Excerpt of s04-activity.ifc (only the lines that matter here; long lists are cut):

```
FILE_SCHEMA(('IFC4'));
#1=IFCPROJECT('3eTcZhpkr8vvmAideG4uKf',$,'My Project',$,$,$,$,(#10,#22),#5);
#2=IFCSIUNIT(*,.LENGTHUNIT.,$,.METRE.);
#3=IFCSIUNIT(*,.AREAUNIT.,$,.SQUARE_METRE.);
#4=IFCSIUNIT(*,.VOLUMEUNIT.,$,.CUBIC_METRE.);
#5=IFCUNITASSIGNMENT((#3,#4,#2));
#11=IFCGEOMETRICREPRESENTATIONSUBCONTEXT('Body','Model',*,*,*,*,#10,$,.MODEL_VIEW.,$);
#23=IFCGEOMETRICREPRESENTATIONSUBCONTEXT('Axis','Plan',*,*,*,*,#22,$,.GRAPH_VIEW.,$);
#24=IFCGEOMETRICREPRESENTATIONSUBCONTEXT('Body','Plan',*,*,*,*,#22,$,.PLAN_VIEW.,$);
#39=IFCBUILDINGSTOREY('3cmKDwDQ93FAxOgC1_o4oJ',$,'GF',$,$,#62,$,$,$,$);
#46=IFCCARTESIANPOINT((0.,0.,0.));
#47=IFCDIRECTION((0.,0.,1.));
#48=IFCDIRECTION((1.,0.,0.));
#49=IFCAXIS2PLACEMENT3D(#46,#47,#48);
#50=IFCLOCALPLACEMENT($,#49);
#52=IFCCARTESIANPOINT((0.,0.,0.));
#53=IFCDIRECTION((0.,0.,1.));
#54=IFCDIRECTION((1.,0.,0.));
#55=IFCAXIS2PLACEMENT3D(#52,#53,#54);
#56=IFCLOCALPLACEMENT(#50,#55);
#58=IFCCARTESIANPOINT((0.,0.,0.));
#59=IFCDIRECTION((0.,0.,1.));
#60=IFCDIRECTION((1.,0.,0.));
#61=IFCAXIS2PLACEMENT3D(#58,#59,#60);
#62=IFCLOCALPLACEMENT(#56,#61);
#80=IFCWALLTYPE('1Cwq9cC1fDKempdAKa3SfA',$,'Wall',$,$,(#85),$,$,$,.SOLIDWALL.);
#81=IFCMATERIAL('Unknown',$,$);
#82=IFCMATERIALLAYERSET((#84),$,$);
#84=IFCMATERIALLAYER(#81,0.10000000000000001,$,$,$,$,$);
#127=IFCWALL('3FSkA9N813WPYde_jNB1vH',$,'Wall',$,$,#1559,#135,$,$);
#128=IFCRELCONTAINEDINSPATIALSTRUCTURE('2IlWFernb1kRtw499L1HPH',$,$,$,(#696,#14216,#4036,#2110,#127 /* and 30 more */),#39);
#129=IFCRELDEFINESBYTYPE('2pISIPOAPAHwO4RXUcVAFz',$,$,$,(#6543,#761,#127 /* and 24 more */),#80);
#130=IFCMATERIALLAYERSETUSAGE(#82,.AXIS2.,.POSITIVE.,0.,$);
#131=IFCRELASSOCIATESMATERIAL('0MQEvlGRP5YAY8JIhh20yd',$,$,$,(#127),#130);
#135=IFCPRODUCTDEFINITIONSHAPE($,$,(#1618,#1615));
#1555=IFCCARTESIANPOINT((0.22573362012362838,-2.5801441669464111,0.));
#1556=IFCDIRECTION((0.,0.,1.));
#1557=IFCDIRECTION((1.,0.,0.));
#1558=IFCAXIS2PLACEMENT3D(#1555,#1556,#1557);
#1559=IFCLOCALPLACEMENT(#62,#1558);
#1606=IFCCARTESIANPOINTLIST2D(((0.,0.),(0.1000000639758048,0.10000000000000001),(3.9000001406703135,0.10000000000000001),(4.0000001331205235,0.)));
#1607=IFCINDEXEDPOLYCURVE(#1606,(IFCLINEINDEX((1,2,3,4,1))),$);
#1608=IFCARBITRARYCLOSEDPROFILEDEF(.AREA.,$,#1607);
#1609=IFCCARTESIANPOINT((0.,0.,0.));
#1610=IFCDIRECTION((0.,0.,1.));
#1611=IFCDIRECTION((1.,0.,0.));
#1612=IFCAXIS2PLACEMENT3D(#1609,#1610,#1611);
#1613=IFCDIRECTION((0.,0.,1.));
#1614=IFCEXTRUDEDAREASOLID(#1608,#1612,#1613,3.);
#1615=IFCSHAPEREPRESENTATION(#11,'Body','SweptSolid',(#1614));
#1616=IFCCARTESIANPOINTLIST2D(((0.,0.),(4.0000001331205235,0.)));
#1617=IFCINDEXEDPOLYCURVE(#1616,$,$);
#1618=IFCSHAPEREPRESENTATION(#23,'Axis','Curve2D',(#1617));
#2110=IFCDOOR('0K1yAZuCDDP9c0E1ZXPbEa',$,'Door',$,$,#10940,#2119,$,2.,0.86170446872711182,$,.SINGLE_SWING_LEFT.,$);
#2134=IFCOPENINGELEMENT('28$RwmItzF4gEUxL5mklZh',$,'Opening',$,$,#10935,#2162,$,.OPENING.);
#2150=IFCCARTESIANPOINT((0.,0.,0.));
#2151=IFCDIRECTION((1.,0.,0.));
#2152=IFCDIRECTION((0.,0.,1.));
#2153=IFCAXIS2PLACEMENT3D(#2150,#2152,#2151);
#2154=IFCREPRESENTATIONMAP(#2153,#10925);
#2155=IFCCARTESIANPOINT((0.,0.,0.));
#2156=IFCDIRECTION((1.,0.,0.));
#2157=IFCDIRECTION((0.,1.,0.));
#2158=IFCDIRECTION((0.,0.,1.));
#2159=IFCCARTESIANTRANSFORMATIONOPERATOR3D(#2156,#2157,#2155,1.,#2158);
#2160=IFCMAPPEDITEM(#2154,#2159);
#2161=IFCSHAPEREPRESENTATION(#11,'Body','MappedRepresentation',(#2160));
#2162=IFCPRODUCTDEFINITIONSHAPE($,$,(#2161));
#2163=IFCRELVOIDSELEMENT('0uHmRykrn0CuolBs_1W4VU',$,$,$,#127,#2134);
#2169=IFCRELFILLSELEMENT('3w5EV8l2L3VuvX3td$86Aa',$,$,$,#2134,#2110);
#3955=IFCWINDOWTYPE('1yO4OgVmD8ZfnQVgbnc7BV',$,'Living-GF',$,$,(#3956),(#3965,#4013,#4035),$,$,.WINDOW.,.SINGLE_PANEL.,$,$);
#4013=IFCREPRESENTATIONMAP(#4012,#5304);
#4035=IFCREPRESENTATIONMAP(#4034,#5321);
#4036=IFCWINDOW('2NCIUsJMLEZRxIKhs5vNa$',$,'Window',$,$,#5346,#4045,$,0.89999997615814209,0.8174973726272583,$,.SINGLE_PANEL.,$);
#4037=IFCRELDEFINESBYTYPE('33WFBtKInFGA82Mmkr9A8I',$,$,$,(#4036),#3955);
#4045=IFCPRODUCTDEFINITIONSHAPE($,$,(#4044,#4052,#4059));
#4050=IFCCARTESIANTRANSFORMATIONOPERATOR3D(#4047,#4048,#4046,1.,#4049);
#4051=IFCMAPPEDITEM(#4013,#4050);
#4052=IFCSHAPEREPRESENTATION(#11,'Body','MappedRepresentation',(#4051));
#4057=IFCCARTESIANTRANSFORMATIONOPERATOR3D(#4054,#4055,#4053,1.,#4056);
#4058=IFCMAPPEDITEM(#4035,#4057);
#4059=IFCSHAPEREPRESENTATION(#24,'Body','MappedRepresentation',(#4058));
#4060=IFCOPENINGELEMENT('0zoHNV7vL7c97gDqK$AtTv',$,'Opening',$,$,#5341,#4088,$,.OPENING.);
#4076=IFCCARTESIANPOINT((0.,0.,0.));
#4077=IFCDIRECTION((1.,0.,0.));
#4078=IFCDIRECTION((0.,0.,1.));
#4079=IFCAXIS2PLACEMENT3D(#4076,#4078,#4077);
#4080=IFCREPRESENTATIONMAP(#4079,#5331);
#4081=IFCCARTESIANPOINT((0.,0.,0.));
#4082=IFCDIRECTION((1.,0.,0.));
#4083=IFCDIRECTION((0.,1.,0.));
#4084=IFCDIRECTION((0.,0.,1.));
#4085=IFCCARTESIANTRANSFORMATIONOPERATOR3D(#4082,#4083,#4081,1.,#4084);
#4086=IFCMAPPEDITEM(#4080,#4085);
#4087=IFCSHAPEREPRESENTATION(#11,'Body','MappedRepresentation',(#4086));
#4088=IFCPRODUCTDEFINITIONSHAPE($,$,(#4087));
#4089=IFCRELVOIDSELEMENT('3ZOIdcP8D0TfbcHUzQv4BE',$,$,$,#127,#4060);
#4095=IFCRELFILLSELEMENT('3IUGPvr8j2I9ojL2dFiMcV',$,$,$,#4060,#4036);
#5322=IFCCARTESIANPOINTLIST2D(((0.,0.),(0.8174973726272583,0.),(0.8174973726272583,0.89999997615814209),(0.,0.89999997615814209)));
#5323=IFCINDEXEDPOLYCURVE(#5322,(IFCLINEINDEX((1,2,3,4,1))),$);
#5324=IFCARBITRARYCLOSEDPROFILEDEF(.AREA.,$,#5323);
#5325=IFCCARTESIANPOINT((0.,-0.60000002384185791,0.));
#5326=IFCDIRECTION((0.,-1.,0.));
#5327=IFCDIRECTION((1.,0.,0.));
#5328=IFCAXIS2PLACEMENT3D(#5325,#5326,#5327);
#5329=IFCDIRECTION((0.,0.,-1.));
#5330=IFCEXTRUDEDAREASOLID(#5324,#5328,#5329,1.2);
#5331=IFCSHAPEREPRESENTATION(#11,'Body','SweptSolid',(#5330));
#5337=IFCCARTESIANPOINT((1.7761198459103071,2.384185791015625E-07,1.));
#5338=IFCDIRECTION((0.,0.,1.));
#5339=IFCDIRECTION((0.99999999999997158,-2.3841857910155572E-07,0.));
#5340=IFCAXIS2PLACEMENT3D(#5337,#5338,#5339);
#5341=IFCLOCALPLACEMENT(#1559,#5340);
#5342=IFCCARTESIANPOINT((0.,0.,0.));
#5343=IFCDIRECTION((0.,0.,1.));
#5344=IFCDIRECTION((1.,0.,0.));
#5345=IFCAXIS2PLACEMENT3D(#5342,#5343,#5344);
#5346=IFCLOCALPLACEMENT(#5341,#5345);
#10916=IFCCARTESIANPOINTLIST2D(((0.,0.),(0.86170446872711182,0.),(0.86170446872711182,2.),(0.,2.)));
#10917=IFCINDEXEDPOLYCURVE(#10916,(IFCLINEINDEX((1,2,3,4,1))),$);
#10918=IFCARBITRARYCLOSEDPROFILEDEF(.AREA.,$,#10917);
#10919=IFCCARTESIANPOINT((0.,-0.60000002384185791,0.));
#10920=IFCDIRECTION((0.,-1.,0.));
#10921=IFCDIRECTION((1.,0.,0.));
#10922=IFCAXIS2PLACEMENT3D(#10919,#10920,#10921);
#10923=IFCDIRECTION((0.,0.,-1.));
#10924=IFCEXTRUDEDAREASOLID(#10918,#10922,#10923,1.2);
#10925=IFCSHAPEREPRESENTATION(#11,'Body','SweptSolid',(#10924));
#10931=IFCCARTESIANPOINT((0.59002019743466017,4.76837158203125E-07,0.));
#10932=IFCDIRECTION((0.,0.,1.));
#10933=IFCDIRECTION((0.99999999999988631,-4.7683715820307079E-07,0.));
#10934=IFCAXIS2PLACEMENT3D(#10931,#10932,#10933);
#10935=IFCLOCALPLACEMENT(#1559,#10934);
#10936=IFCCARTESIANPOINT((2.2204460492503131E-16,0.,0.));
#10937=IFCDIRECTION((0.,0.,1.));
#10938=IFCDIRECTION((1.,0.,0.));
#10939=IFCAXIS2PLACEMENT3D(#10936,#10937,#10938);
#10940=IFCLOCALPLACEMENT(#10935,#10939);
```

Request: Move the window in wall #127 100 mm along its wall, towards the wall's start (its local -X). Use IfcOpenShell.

```python
import ifcopenshell
import ifcopenshell.api.geometry
import ifcopenshell.util.placement

model = ifcopenshell.open("s04-activity.ifc")

window = model.by_id(4036)
opening = window.FillsVoids[0].RelatingOpeningElement
wall = opening.VoidsElements[0].RelatingBuildingElement

wall_matrix = ifcopenshell.util.placement.get_local_placement(wall.ObjectPlacement)
shift = wall_matrix[:3, 0] * -0.1
before = ifcopenshell.util.placement.get_local_placement(window.ObjectPlacement)[:3, 3].copy()

# The window is placed relative to its opening, so it follows when the opening moves.
matrix = ifcopenshell.util.placement.get_local_placement(opening.ObjectPlacement)
matrix[:3, 3] += shift
ifcopenshell.api.geometry.edit_object_placement(
    model, product=opening, matrix=matrix, is_si=False, should_transform_children=True
)

after = ifcopenshell.util.placement.get_local_placement(window.ObjectPlacement)[:3, 3]
print("window moved by", (after - before).round(3) + 0.0)

model.write("s04-activity_rev.ifc")
```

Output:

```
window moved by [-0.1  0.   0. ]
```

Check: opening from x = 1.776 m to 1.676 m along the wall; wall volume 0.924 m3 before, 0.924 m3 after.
